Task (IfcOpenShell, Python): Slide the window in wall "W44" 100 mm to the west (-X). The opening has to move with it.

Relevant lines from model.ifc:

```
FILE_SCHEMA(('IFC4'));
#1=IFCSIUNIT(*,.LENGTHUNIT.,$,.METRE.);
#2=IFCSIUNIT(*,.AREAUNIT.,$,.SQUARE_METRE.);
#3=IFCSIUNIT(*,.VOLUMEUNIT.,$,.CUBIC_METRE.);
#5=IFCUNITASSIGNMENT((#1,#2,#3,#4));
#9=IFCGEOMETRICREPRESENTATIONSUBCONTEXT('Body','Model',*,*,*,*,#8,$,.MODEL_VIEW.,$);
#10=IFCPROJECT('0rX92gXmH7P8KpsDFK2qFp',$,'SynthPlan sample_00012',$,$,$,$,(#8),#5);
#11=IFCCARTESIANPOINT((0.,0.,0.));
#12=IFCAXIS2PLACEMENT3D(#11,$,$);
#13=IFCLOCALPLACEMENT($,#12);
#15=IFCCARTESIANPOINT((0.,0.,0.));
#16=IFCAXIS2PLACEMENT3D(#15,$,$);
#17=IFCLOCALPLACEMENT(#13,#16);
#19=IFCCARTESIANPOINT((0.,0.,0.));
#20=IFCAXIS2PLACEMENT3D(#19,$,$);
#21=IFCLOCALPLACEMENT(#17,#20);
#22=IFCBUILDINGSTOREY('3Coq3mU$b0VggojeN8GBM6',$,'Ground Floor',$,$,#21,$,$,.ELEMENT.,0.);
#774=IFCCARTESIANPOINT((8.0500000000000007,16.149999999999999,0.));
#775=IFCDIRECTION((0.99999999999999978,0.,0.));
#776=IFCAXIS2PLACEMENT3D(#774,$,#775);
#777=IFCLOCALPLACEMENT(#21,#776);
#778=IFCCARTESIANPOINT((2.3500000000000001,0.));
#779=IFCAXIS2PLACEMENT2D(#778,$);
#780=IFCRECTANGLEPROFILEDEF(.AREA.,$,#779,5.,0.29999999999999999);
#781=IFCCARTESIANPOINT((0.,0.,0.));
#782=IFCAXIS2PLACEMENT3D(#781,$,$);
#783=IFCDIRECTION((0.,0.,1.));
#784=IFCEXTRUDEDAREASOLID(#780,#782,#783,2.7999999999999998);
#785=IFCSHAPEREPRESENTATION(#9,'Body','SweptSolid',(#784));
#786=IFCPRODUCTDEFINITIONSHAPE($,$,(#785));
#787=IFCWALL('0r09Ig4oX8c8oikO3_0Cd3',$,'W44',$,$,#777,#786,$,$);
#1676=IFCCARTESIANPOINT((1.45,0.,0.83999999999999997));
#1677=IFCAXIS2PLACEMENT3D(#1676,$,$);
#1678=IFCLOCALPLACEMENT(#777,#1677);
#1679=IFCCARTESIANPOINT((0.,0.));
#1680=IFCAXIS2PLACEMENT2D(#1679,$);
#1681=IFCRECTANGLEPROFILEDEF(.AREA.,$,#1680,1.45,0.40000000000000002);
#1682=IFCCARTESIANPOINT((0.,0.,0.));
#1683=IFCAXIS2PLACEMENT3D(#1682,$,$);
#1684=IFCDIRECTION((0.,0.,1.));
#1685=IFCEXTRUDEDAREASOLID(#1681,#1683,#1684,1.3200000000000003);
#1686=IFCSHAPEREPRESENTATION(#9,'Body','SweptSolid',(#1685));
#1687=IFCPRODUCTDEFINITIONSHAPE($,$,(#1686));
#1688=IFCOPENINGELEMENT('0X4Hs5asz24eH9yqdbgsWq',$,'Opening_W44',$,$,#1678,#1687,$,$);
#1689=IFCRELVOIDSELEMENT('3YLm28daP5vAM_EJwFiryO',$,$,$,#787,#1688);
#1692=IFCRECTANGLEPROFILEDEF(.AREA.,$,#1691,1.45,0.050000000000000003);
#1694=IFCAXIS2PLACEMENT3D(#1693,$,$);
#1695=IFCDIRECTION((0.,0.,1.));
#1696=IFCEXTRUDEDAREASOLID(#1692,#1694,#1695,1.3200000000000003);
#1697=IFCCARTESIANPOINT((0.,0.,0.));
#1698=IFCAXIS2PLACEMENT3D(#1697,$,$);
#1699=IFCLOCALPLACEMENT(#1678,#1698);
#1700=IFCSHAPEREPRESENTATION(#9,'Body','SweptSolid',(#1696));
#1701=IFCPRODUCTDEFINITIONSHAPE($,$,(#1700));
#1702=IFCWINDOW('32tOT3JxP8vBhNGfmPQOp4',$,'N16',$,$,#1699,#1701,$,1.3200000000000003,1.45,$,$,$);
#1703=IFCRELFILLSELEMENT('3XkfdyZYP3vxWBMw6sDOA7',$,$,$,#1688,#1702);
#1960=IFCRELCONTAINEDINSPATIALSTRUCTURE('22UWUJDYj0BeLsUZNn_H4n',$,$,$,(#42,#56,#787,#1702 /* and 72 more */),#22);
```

```python
import ifcopenshell
import ifcopenshell.api.geometry
import ifcopenshell.util.placement

model = ifcopenshell.open("model.ifc")

window = model.by_guid("32tOT3JxP8vBhNGfmPQOp4")
opening = window.FillsVoids[0].RelatingOpeningElement
wall = opening.VoidsElements[0].RelatingBuildingElement

wall_matrix = ifcopenshell.util.placement.get_local_placement(wall.ObjectPlacement)
shift = wall_matrix[:3, 0] * -0.1
before = ifcopenshell.util.placement.get_local_placement(window.ObjectPlacement)[:3, 3].copy()

# The window is placed relative to its opening, so it follows when the opening moves.
matrix = ifcopenshell.util.placement.get_local_placement(opening.ObjectPlacement)
matrix[:3, 3] += shift
ifcopenshell.api.geometry.edit_object_placement(
    model, product=opening, matrix=matrix, is_si=False, should_transform_children=True
)

after = ifcopenshell.util.placement.get_local_placement(window.ObjectPlacement)[:3, 3]
print("window moved by", (after - before).round(3) + 0.0)

model.write("model-out.ifc")
```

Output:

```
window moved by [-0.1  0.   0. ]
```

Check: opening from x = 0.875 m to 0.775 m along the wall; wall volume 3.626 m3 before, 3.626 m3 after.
